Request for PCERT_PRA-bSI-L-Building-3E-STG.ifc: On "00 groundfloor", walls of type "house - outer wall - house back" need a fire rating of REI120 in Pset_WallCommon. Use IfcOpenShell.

First a look at what the model holds.

```python
import ifcopenshell
import ifcopenshell.util.element

model = ifcopenshell.open("PCERT_PRA-bSI-L-Building-3E-STG.ifc")
print(model.schema)
storey = next(s for s in model.by_type("IfcBuildingStorey") if s.Name == "00 groundfloor")
walls = [e for e in ifcopenshell.util.element.get_decomposition(storey) if e.is_a("IfcWall")]
seen = {}
for e in walls:
    element_type = ifcopenshell.util.element.get_type(e)
    key = (element_type.Name if element_type != e and element_type else None, ifcopenshell.util.element.get_pset(e, "Pset_WallCommon", "FireRating"))
    seen[key] = seen.get(key, 0) + 1
for (name, value), count in sorted(seen.items(), key=str):
    print(count, "x", name, "|", value)
```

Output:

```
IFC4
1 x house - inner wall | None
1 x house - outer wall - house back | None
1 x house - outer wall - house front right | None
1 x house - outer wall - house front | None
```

```python
import ifcopenshell
import ifcopenshell.api.pset
import ifcopenshell.util.element

model = ifcopenshell.open("PCERT_PRA-bSI-L-Building-3E-STG.ifc")

storey = next(s for s in model.by_type("IfcBuildingStorey") if s.Name == "00 groundfloor")
walls = [e for e in ifcopenshell.util.element.get_decomposition(storey) if e.is_a("IfcWall")]

count = 0
for e in walls:
    element_type = ifcopenshell.util.element.get_type(e)
    if element_type in (None, e) or element_type.Name != "house - outer wall - house back":
        continue
    # add_pset returns the element's existing set when there is one.
    pset = ifcopenshell.api.pset.add_pset(model, product=e, name="Pset_WallCommon")
    ifcopenshell.api.pset.edit_pset(model, pset=pset, properties={"FireRating": "REI120"})
    count += 1

print(count, "walls updated")

model.write("PCERT_PRA-bSI-L-Building-3E-STG_updated.ifc")
```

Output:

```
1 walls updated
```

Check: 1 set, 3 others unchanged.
